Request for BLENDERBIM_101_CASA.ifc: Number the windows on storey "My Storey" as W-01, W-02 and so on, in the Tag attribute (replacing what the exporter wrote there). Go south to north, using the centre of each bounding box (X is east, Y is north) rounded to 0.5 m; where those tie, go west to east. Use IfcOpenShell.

First a look at what the model holds.

```python
import ifcopenshell
import ifcopenshell.util.element
import ifcopenshell.util.placement

model = ifcopenshell.open("BLENDERBIM_101_CASA.ifc")
print(model.schema)
storey = next(s for s in model.by_type("IfcBuildingStorey") if s.Name == "My Storey")
windows = [e for e in ifcopenshell.util.element.get_decomposition(storey) if e.is_a("IfcWindow")]
for e in sorted(windows, key=lambda e: e.id()):
    origin = ifcopenshell.util.placement.get_local_placement(e.ObjectPlacement)[:3, 3]
    print(e.id(), e.Tag, e.Name, origin.round(2) + 0.0, sep=" | ")
```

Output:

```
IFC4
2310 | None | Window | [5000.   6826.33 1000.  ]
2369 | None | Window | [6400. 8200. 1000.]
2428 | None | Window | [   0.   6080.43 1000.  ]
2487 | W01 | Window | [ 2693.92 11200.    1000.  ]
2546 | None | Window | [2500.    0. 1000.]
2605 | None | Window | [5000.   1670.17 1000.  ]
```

```python
import ifcopenshell
import ifcopenshell.geom
import ifcopenshell.util.element
import ifcopenshell.util.shape

model = ifcopenshell.open("BLENDERBIM_101_CASA.ifc")
settings = ifcopenshell.geom.settings()
settings.set("use-world-coords", True)


def centre(element):
    shape = ifcopenshell.geom.create_shape(settings, element)
    return ifcopenshell.util.shape.get_bbox_centroid(shape.geometry)


storey = next(s for s in model.by_type("IfcBuildingStorey") if s.Name == "My Storey")
windows = [e for e in ifcopenshell.util.element.get_decomposition(storey) if e.is_a("IfcWindow")]

# Insertion points can sit at a corner or the storey origin, so sort by the geometry (in metres).
centres = {e: centre(e) for e in windows}
windows.sort(key=lambda e: (round(centres[e][1] / 0.5), centres[e][0]))

for i, e in enumerate(windows, start=1):
    number = f"W-{i:02d}"
    e.Tag = number
    print(e.id(), number)

model.write("BLENDERBIM_101_CASA_rev.ifc")
```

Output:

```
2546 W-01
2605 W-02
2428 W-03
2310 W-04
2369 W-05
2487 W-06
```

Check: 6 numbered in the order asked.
